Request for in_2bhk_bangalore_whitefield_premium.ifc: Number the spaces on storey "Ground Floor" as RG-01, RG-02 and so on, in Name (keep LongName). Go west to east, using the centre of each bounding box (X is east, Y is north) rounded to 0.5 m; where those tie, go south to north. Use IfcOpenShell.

First a look at what the model holds.

```python
import ifcopenshell
import ifcopenshell.util.element
import ifcopenshell.util.placement

model = ifcopenshell.open("in_2bhk_bangalore_whitefield_premium.ifc")
print(model.schema)
storey = next(s for s in model.by_type("IfcBuildingStorey") if s.Name == "Ground Floor")
spaces = [e for e in ifcopenshell.util.element.get_decomposition(storey) if e.is_a("IfcSpace")]
for e in sorted(spaces, key=lambda e: e.id()):
    origin = ifcopenshell.util.placement.get_local_placement(e.ObjectPlacement)[:3, 3]
    print(e.id(), e.Name, e.LongName, origin.round(2) + 0.0, sep=" | ")
```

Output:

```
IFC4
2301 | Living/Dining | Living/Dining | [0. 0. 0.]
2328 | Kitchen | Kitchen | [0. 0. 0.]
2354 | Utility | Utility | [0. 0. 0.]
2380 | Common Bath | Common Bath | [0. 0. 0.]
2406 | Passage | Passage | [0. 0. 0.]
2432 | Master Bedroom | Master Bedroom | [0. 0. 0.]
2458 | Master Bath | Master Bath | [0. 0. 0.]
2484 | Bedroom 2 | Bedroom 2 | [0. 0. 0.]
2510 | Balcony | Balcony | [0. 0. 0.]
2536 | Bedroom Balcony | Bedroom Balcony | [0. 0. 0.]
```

```python
import ifcopenshell
import ifcopenshell.geom
import ifcopenshell.util.element
import ifcopenshell.util.shape

model = ifcopenshell.open("in_2bhk_bangalore_whitefield_premium.ifc")
settings = ifcopenshell.geom.settings()
settings.set("use-world-coords", True)


def centre(element):
    shape = ifcopenshell.geom.create_shape(settings, element)
    return ifcopenshell.util.shape.get_bbox_centroid(shape.geometry)


storey = next(s for s in model.by_type("IfcBuildingStorey") if s.Name == "Ground Floor")
spaces = [e for e in ifcopenshell.util.element.get_decomposition(storey) if e.is_a("IfcSpace")]

# Insertion points can sit at a corner or the storey origin, so sort by the geometry (in metres).
centres = {e: centre(e) for e in spaces}
spaces.sort(key=lambda e: (round(centres[e][0] / 0.5), centres[e][1]))

for i, e in enumerate(spaces, start=1):
    number = f"RG-{i:02d}"
    e.Name = number
    print(e.id(), number)

model.write("in_2bhk_bangalore_whitefield_premium_updated.ifc")
```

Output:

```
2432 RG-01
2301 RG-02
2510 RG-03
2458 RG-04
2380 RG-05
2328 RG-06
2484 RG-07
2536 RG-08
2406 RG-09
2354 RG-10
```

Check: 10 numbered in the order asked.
